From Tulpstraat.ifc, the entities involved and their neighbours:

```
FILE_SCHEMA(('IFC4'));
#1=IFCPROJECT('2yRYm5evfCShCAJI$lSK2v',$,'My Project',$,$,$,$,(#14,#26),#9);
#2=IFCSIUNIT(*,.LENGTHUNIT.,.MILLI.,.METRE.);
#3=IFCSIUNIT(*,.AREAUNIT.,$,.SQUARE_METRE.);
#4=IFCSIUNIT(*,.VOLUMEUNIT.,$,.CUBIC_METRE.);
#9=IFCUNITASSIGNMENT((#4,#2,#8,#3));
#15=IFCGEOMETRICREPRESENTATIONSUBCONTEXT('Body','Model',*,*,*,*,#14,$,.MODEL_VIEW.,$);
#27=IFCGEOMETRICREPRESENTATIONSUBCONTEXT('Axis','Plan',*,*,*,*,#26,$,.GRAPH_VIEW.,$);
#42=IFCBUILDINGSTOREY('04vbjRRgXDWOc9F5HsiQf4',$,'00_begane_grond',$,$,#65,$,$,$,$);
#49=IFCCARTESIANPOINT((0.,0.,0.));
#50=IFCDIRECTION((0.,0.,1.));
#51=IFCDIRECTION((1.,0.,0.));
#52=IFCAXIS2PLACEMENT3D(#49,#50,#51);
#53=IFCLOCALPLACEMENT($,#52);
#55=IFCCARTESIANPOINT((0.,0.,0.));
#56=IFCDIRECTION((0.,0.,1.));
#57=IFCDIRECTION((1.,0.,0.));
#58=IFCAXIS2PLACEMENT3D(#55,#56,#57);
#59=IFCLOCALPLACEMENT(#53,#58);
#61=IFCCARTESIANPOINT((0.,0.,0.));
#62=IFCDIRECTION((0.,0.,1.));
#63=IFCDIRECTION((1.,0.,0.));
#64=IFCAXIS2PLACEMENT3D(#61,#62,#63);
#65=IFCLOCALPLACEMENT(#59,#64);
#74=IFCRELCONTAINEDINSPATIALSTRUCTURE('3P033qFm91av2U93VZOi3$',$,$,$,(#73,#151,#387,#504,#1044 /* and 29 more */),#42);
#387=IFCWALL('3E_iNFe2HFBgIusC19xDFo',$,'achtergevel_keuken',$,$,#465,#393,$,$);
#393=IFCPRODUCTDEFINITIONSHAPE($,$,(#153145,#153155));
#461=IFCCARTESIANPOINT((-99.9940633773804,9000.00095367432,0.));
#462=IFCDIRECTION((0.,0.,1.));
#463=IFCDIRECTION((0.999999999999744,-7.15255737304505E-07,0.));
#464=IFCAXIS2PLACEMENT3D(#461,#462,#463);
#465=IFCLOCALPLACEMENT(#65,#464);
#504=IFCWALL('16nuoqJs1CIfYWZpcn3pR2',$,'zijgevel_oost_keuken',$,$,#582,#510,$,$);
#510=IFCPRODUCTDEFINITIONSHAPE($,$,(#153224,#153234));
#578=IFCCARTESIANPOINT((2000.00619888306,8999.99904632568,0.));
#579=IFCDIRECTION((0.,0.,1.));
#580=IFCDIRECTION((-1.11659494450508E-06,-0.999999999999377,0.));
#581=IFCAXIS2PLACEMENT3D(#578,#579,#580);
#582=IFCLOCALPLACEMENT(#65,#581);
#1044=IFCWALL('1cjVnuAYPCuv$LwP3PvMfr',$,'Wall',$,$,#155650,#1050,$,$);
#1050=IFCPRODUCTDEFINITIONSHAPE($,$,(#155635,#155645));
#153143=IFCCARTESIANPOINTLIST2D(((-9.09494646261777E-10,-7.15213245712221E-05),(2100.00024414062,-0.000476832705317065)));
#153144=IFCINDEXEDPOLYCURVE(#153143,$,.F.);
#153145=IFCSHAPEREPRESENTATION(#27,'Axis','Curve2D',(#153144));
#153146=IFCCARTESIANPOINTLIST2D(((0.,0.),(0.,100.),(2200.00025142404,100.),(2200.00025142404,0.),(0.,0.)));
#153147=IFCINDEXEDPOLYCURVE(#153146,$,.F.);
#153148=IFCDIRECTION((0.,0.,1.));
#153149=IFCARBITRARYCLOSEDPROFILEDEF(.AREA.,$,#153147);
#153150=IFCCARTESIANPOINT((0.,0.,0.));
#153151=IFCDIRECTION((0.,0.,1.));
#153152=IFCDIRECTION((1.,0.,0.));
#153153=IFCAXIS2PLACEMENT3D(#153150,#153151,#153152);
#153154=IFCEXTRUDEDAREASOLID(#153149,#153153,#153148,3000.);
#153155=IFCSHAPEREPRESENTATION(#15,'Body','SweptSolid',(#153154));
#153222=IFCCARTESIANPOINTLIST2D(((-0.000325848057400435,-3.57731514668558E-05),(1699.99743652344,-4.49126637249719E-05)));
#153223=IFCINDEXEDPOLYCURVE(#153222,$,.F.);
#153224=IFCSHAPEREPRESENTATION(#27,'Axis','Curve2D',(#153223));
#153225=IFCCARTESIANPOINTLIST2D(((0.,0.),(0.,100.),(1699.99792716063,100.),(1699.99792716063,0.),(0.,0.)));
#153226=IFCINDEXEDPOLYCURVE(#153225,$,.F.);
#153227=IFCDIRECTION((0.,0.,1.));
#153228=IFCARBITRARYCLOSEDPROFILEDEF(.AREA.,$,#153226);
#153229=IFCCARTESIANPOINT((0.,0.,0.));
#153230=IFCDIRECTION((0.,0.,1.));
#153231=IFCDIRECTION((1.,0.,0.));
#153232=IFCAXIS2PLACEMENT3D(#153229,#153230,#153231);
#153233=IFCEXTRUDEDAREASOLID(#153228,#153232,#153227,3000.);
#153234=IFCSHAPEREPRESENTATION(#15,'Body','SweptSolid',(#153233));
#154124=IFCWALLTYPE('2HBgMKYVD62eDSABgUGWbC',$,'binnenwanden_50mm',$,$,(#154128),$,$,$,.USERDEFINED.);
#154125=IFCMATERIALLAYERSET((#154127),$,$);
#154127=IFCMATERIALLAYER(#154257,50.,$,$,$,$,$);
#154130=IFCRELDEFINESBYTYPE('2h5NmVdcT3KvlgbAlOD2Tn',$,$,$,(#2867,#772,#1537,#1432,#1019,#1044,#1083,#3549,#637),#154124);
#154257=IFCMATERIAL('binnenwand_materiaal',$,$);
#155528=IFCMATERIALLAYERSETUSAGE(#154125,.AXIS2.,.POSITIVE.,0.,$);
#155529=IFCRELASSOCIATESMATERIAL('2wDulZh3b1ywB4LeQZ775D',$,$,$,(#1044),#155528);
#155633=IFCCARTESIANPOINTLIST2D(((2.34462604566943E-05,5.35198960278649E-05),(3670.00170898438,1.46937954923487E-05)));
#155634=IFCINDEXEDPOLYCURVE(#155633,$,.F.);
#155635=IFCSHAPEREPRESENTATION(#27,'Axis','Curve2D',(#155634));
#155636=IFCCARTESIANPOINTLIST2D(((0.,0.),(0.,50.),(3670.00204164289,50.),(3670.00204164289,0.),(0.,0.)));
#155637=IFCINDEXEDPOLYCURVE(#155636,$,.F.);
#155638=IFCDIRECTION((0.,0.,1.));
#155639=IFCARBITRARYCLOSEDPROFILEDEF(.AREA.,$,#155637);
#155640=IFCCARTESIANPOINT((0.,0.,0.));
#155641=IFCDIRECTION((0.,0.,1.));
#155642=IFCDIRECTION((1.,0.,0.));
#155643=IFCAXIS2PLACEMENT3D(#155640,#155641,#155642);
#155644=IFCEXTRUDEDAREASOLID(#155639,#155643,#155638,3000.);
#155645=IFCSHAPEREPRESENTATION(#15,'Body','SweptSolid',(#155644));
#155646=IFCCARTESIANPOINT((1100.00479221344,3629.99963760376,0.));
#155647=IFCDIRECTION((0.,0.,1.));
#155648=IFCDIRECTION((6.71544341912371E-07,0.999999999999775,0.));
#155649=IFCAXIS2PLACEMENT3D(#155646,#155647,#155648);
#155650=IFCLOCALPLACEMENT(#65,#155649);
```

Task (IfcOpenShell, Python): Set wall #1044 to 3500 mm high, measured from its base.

```python
import ifcopenshell
import ifcopenshell.geom
import ifcopenshell.util.representation
import ifcopenshell.util.shape
import ifcopenshell.util.unit

model = ifcopenshell.open("Tulpstraat.ifc")
unit_scale = ifcopenshell.util.unit.calculate_unit_scale(model)
settings = ifcopenshell.geom.settings()


def volume(element):
    """Net volume in cubic metres, openings subtracted."""
    shape = ifcopenshell.geom.create_shape(settings, element)
    return ifcopenshell.util.shape.get_volume(shape.geometry)


wall = model.by_guid("1cjVnuAYPCuv$LwP3PvMfr")
before = volume(wall)

body = ifcopenshell.util.representation.get_representation(wall, "Model", "Body")
solid = body.Items[0]
old_height = solid.Depth
solid.Depth = 3.5 / unit_scale
after = volume(wall)

print(f"height {old_height:g} -> {solid.Depth:g}, volume {before:.3f} -> {after:.3f} m3")

model.write("Tulpstraat-out.ifc")
```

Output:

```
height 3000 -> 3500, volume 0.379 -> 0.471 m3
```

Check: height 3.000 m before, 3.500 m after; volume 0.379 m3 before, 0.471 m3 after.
